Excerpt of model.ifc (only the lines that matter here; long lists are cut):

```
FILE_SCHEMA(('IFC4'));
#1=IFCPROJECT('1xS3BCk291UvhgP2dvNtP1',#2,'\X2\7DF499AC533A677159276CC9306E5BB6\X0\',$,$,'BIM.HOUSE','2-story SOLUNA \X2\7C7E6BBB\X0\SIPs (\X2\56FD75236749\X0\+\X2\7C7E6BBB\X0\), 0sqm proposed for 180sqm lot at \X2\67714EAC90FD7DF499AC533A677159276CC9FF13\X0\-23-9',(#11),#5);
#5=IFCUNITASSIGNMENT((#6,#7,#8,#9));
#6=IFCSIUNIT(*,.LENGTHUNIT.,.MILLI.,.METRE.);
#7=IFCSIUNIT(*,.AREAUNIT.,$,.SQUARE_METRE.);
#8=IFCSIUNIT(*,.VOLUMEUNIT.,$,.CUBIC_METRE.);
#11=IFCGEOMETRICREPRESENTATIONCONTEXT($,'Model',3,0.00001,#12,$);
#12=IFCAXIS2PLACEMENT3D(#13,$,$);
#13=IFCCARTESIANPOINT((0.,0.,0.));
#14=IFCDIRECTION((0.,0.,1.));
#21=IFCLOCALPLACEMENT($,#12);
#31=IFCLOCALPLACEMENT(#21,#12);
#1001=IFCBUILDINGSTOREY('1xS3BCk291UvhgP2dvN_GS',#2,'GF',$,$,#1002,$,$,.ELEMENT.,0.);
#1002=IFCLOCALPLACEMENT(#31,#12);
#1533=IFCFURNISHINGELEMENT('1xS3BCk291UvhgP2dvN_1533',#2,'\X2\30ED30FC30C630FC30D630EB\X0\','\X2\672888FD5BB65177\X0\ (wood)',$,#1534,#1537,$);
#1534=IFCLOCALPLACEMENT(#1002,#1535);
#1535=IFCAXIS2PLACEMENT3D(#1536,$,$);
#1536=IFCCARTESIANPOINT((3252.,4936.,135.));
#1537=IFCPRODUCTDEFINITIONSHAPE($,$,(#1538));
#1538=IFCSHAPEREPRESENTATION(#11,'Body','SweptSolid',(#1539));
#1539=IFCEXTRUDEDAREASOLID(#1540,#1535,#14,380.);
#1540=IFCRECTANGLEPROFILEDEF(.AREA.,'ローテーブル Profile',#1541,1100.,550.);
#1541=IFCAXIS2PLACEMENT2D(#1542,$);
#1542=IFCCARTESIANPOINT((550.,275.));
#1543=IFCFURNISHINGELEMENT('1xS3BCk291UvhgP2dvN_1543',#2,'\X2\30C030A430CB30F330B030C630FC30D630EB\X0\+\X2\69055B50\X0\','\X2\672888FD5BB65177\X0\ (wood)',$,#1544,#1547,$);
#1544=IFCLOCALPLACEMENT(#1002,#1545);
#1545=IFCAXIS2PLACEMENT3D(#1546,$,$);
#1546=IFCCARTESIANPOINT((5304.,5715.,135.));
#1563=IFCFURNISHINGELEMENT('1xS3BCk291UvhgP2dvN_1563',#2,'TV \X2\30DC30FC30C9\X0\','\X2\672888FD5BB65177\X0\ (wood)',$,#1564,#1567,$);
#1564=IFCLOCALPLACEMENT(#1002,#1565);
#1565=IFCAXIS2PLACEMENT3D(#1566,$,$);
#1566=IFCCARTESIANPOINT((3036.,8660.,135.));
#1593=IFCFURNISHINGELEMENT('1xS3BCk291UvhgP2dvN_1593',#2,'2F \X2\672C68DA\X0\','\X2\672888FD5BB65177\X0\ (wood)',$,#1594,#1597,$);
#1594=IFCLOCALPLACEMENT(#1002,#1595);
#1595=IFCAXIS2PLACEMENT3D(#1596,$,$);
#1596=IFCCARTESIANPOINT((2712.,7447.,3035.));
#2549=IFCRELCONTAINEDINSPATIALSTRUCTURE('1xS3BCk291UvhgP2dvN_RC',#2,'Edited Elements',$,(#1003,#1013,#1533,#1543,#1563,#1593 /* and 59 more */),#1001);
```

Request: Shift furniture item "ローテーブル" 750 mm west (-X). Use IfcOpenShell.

```python
import ifcopenshell
import ifcopenshell.api.geometry
import ifcopenshell.util.placement

model = ifcopenshell.open("model.ifc")

item = model.by_id(1533)
matrix = ifcopenshell.util.placement.get_local_placement(item.ObjectPlacement)
matrix[0, 3] -= 750.0
ifcopenshell.api.geometry.edit_object_placement(model, product=item, matrix=matrix, is_si=False)

print(ifcopenshell.util.placement.get_local_placement(item.ObjectPlacement).round(3) + 0.0)

model.write("model-out.ifc")
```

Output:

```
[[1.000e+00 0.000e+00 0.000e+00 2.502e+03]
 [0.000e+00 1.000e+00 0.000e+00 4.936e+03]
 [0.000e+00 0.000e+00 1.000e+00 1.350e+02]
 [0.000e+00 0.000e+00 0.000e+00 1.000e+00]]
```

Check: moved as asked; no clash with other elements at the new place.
